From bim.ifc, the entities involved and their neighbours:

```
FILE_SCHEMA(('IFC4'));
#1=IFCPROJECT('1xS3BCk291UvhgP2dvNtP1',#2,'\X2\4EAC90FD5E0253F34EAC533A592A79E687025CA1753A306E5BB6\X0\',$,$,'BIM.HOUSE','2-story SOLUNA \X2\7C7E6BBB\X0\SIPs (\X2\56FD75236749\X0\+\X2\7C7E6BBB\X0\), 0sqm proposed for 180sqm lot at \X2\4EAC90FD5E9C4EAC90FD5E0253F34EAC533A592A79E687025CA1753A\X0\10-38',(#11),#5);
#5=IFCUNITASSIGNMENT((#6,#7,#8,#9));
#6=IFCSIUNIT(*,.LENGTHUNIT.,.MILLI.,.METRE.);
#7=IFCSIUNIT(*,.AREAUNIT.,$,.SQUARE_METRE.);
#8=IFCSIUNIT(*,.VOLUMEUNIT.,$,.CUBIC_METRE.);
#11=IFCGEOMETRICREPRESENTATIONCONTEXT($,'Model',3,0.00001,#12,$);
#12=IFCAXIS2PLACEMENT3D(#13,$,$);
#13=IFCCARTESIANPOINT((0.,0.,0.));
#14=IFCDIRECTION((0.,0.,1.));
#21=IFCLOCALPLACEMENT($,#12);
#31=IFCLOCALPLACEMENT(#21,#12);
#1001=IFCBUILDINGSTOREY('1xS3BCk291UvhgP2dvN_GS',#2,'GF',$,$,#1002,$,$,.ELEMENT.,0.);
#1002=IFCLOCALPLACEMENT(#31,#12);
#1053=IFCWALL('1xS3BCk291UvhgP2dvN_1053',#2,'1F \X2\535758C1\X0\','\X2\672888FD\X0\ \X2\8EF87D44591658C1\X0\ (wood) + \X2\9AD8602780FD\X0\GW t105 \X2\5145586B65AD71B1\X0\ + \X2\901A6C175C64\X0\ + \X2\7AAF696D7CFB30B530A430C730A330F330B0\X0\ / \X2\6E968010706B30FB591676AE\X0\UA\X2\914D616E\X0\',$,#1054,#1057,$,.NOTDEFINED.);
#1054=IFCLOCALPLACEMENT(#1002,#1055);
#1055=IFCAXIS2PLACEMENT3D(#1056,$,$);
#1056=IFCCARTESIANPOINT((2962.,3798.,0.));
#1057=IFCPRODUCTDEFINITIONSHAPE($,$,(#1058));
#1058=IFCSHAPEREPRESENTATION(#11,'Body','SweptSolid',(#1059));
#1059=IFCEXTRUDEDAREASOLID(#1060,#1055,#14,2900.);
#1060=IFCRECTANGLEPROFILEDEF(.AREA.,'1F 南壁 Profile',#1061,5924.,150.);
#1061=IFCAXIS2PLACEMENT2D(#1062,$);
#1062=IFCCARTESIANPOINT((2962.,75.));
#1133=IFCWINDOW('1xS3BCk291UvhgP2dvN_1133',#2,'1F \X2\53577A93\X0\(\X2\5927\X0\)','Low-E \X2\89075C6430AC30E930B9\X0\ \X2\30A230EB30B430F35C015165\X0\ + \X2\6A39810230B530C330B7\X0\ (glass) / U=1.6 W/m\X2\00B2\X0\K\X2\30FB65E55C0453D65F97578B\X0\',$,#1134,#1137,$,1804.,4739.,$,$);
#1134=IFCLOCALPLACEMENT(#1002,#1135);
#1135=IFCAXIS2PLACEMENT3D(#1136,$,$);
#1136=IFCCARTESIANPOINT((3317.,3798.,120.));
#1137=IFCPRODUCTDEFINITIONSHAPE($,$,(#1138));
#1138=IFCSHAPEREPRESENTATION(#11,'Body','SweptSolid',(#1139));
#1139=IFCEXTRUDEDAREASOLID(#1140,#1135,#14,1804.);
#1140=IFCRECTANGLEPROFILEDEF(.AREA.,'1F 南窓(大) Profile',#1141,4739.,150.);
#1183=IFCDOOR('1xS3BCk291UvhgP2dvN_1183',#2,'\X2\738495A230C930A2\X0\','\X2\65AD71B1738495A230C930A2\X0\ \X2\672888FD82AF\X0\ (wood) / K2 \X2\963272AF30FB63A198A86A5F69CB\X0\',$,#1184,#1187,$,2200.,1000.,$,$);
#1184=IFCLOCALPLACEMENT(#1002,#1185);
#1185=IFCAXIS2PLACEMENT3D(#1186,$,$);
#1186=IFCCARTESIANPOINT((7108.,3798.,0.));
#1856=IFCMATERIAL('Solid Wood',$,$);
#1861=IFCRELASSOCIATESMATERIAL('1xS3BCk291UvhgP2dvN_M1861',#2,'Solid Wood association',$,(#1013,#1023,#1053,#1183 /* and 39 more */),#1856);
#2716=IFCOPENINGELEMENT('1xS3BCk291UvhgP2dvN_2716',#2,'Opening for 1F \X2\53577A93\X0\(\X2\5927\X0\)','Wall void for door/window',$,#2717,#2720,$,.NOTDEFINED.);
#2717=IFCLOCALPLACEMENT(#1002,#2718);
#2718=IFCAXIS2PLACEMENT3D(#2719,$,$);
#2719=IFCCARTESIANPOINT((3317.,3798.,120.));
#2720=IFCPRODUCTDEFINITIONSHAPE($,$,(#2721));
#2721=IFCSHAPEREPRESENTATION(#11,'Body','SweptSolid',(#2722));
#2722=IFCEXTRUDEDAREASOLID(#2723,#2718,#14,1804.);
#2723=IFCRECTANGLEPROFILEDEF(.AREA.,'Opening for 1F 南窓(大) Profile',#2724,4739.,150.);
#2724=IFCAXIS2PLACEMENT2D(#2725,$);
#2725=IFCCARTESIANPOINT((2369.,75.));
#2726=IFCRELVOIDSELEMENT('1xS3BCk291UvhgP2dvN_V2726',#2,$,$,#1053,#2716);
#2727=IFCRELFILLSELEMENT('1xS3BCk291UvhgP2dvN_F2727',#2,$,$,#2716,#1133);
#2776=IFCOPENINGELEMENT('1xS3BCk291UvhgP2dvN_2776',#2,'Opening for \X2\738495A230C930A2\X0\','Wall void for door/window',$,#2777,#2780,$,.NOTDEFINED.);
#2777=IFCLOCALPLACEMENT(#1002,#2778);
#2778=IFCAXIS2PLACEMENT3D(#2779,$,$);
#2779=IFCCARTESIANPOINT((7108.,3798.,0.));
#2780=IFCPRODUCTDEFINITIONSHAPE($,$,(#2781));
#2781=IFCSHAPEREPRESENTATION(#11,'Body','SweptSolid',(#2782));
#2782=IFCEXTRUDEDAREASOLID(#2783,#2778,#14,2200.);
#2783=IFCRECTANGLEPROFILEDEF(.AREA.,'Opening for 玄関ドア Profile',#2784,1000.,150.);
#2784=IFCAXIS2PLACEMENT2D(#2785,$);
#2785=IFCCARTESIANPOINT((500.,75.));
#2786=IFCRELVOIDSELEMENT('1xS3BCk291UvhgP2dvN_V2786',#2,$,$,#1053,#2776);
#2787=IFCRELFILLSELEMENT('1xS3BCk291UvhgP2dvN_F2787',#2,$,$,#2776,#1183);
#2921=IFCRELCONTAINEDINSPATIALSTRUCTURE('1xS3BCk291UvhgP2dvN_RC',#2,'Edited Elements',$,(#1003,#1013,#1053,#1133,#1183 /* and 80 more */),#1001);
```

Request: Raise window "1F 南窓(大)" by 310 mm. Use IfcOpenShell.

```python
import numpy as np
import ifcopenshell
import ifcopenshell.api.geometry
import ifcopenshell.util.placement
import ifcopenshell.util.unit

model = ifcopenshell.open("bim.ifc")
unit_scale = ifcopenshell.util.unit.calculate_unit_scale(model)

window = model.by_guid("1xS3BCk291UvhgP2dvN_1133")
opening = window.FillsVoids[0].RelatingOpeningElement
dz = 0.31 / unit_scale

shift = np.array([0.0, 0.0, dz])
# The window is not placed relative to its opening, so move both.
for product in (opening, window):
    matrix = ifcopenshell.util.placement.get_local_placement(product.ObjectPlacement)
    matrix[:3, 3] += shift
    ifcopenshell.api.geometry.edit_object_placement(model, product=product, matrix=matrix, is_si=False)

print(f"moved by {dz * unit_scale:+.3f} m")

model.write("bim_updated.ifc")
```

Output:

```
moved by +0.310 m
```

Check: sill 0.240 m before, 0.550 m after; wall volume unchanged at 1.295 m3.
